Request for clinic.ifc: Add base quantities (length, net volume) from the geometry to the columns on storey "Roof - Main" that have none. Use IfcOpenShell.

First a look at what the model holds.

```python
import ifcopenshell
import ifcopenshell.util.element
import ifcopenshell.util.unit

model = ifcopenshell.open("clinic.ifc")
print(model.schema)
for unit_type in ("LENGTHUNIT", "AREAUNIT", "VOLUMEUNIT"):
    print(unit_type, ifcopenshell.util.unit.calculate_unit_scale(model, unit_type))
storey = next(s for s in model.by_type("IfcBuildingStorey") if s.Name == "Roof - Main")
columns = [e for e in ifcopenshell.util.element.get_decomposition(storey) if e.is_a("IfcColumn")]
for e in sorted(columns, key=lambda e: e.id()):
    print(e.id(), e.is_a(), e.Name, list(ifcopenshell.util.element.get_psets(e, qtos_only=True)), sep=" | ")
```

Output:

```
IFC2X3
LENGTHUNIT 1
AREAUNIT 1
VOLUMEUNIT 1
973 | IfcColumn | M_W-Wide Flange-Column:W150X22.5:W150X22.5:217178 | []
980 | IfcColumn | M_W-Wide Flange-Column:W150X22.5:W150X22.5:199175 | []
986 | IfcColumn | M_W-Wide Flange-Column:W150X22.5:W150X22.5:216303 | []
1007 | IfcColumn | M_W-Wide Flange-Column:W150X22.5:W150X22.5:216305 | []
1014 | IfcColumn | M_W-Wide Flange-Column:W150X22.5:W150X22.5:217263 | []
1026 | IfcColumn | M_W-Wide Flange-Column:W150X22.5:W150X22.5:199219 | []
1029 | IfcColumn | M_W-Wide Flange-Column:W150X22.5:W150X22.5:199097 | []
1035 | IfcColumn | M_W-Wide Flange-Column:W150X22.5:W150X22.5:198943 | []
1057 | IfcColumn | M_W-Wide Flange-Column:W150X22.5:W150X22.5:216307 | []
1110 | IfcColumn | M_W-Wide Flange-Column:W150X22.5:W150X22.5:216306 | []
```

```python
import ifcopenshell
import ifcopenshell.api.pset
import ifcopenshell.geom
import ifcopenshell.util.element
import ifcopenshell.util.shape
import ifcopenshell.util.unit

model = ifcopenshell.open("clinic.ifc")
unit_scale = ifcopenshell.util.unit.calculate_unit_scale(model)
volume_scale = ifcopenshell.util.unit.calculate_unit_scale(model, "VOLUMEUNIT")
settings = ifcopenshell.geom.settings()

storey = next(s for s in model.by_type("IfcBuildingStorey") if s.Name == "Roof - Main")
columns = [e for e in ifcopenshell.util.element.get_decomposition(storey) if e.is_a("IfcColumn")]

for e in sorted(columns, key=lambda e: e.id()):
    if ifcopenshell.util.element.get_psets(e, qtos_only=True, should_inherit=False):
        continue
    # Geometry comes back in metres, in the element's own axes.
    shape = ifcopenshell.geom.create_shape(settings, e)
    values = {
        "Length": ifcopenshell.util.shape.get_z(shape.geometry) / unit_scale,
        "NetVolume": ifcopenshell.util.shape.get_volume(shape.geometry) / volume_scale,
    }
    qto = ifcopenshell.api.pset.add_qto(model, product=e, name="BaseQuantities")
    ifcopenshell.api.pset.edit_qto(model, qto=qto, properties=values)
    print(e.id(), {k: round(v, 3) for k, v in values.items()})

model.write("clinic_edited.ifc")
```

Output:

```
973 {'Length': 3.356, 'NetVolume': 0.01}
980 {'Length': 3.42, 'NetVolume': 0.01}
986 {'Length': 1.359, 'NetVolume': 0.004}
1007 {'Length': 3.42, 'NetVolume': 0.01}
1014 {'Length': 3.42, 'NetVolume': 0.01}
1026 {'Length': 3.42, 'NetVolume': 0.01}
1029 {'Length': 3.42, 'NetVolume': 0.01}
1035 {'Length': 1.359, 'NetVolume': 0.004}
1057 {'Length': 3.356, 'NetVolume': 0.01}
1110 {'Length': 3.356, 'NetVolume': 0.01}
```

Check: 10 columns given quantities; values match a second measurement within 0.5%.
